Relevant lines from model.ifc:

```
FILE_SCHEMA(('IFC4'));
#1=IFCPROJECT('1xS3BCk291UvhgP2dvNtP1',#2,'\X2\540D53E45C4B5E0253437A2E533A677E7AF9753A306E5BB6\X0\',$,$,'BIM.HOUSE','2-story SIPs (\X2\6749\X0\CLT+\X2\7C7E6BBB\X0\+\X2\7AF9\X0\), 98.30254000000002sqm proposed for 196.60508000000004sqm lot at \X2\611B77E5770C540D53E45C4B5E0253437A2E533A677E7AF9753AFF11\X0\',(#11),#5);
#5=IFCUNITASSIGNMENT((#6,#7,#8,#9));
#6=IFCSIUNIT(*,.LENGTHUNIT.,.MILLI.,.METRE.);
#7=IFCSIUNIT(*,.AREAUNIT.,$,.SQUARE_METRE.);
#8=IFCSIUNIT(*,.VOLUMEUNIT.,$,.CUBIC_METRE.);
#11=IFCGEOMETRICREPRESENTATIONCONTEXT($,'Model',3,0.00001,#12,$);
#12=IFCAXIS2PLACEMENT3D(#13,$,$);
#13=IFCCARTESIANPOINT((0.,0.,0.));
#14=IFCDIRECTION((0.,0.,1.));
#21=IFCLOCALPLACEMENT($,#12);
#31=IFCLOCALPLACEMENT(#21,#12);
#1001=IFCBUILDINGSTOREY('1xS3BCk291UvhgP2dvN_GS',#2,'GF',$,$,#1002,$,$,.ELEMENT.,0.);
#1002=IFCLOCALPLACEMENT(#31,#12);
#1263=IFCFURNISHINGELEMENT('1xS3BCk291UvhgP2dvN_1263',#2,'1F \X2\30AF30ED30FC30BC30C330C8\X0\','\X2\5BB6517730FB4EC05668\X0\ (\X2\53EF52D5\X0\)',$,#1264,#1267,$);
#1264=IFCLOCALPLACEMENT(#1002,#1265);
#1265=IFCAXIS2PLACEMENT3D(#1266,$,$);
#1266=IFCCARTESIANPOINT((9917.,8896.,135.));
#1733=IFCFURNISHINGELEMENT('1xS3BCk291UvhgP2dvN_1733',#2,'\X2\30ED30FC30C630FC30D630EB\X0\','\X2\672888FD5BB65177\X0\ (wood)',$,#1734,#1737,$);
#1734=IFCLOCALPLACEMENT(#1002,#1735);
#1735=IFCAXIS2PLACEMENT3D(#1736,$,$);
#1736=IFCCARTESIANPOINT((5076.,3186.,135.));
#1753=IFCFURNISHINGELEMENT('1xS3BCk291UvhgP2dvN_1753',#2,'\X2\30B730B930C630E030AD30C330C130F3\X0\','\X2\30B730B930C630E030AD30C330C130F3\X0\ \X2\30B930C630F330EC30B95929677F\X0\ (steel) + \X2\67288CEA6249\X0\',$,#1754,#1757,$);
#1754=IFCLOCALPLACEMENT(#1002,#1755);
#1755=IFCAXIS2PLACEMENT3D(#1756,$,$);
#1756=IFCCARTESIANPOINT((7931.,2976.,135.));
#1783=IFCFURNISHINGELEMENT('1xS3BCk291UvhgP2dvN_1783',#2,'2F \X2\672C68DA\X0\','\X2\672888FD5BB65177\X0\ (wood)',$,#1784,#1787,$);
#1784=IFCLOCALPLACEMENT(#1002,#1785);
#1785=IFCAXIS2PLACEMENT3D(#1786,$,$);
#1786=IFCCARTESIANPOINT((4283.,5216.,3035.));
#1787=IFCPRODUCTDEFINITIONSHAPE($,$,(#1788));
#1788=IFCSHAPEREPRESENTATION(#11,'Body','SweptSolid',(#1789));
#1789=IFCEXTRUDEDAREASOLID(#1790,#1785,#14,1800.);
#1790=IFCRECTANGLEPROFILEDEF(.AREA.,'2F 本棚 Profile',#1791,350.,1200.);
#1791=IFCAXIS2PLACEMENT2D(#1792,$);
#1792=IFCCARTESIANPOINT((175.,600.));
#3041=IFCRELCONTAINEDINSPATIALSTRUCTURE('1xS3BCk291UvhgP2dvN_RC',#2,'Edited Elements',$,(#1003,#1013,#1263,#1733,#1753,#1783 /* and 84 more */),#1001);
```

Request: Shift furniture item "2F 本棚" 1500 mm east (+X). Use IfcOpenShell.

```python
import ifcopenshell
import ifcopenshell.api.geometry
import ifcopenshell.util.placement
import ifcopenshell.util.unit

model = ifcopenshell.open("model.ifc")
unit_scale = ifcopenshell.util.unit.calculate_unit_scale(model)

item = model.by_guid("1xS3BCk291UvhgP2dvN_1783")
matrix = ifcopenshell.util.placement.get_local_placement(item.ObjectPlacement)
matrix[0, 3] += 1.5 / unit_scale
ifcopenshell.api.geometry.edit_object_placement(model, product=item, matrix=matrix, is_si=False)

print(ifcopenshell.util.placement.get_local_placement(item.ObjectPlacement).round(3) + 0.0)

model.write("model_v2.ifc")
```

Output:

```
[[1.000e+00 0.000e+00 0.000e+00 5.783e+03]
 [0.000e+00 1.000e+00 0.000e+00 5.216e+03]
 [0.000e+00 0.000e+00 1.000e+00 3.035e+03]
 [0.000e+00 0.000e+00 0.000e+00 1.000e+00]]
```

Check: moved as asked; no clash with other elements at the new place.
